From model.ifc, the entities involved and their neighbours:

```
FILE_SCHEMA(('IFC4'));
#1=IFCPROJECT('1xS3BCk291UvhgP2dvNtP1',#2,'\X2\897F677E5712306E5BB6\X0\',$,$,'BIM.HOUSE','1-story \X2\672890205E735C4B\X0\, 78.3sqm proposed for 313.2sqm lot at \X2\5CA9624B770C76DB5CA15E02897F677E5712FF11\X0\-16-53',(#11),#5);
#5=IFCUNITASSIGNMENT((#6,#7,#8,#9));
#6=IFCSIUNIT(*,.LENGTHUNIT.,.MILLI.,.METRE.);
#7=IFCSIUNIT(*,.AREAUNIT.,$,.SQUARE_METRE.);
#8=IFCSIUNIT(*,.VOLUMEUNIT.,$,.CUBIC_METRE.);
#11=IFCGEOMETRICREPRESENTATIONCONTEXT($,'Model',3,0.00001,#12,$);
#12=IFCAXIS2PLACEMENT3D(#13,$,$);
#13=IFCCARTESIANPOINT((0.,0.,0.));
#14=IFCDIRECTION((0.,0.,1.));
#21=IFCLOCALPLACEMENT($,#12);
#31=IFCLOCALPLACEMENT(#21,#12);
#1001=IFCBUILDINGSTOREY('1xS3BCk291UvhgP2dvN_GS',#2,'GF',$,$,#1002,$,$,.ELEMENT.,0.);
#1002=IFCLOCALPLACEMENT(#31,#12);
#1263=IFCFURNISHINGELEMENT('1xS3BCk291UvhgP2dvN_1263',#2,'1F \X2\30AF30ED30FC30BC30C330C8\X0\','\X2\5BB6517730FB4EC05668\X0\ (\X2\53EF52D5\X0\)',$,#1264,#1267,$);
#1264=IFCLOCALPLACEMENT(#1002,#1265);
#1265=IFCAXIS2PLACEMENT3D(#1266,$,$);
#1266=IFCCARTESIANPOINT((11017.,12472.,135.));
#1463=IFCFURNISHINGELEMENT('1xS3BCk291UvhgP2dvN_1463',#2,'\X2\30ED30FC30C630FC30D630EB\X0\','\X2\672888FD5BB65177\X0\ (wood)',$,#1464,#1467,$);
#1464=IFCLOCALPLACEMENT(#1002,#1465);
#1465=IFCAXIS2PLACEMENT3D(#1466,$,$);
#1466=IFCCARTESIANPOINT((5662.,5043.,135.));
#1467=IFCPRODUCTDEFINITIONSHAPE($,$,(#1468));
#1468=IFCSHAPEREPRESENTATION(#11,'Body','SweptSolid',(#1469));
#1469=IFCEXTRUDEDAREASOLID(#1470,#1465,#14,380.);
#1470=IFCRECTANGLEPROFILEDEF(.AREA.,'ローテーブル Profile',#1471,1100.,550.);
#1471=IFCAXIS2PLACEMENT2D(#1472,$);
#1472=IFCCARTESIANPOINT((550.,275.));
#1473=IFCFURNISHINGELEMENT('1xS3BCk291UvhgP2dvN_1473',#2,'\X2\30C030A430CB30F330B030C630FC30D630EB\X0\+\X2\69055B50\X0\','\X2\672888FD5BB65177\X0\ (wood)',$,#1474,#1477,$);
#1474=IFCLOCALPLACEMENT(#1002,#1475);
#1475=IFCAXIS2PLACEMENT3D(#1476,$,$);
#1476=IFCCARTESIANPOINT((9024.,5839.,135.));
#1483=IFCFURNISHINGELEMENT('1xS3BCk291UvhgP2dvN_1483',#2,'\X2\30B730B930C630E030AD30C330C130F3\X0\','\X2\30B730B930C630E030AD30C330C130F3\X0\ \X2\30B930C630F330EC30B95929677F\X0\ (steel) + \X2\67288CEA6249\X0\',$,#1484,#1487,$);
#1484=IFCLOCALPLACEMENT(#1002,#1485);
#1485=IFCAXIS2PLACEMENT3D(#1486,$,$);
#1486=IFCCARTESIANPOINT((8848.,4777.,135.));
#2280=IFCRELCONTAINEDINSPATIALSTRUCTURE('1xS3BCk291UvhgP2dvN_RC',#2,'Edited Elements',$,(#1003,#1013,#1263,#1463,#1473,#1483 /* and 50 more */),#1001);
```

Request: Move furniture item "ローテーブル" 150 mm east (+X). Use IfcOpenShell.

```python
import ifcopenshell
import ifcopenshell.api.geometry
import ifcopenshell.util.placement
import ifcopenshell.util.unit

model = ifcopenshell.open("model.ifc")
unit_scale = ifcopenshell.util.unit.calculate_unit_scale(model)

item = model.by_id(1463)
matrix = ifcopenshell.util.placement.get_local_placement(item.ObjectPlacement)
matrix[0, 3] += 0.15 / unit_scale
ifcopenshell.api.geometry.edit_object_placement(model, product=item, matrix=matrix, is_si=False)

print(ifcopenshell.util.placement.get_local_placement(item.ObjectPlacement).round(3) + 0.0)

model.write("model_v2.ifc")
```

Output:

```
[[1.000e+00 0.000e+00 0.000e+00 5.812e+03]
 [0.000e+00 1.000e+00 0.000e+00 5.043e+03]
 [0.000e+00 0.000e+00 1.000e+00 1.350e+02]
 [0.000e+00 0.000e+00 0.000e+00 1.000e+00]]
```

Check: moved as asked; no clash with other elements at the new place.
